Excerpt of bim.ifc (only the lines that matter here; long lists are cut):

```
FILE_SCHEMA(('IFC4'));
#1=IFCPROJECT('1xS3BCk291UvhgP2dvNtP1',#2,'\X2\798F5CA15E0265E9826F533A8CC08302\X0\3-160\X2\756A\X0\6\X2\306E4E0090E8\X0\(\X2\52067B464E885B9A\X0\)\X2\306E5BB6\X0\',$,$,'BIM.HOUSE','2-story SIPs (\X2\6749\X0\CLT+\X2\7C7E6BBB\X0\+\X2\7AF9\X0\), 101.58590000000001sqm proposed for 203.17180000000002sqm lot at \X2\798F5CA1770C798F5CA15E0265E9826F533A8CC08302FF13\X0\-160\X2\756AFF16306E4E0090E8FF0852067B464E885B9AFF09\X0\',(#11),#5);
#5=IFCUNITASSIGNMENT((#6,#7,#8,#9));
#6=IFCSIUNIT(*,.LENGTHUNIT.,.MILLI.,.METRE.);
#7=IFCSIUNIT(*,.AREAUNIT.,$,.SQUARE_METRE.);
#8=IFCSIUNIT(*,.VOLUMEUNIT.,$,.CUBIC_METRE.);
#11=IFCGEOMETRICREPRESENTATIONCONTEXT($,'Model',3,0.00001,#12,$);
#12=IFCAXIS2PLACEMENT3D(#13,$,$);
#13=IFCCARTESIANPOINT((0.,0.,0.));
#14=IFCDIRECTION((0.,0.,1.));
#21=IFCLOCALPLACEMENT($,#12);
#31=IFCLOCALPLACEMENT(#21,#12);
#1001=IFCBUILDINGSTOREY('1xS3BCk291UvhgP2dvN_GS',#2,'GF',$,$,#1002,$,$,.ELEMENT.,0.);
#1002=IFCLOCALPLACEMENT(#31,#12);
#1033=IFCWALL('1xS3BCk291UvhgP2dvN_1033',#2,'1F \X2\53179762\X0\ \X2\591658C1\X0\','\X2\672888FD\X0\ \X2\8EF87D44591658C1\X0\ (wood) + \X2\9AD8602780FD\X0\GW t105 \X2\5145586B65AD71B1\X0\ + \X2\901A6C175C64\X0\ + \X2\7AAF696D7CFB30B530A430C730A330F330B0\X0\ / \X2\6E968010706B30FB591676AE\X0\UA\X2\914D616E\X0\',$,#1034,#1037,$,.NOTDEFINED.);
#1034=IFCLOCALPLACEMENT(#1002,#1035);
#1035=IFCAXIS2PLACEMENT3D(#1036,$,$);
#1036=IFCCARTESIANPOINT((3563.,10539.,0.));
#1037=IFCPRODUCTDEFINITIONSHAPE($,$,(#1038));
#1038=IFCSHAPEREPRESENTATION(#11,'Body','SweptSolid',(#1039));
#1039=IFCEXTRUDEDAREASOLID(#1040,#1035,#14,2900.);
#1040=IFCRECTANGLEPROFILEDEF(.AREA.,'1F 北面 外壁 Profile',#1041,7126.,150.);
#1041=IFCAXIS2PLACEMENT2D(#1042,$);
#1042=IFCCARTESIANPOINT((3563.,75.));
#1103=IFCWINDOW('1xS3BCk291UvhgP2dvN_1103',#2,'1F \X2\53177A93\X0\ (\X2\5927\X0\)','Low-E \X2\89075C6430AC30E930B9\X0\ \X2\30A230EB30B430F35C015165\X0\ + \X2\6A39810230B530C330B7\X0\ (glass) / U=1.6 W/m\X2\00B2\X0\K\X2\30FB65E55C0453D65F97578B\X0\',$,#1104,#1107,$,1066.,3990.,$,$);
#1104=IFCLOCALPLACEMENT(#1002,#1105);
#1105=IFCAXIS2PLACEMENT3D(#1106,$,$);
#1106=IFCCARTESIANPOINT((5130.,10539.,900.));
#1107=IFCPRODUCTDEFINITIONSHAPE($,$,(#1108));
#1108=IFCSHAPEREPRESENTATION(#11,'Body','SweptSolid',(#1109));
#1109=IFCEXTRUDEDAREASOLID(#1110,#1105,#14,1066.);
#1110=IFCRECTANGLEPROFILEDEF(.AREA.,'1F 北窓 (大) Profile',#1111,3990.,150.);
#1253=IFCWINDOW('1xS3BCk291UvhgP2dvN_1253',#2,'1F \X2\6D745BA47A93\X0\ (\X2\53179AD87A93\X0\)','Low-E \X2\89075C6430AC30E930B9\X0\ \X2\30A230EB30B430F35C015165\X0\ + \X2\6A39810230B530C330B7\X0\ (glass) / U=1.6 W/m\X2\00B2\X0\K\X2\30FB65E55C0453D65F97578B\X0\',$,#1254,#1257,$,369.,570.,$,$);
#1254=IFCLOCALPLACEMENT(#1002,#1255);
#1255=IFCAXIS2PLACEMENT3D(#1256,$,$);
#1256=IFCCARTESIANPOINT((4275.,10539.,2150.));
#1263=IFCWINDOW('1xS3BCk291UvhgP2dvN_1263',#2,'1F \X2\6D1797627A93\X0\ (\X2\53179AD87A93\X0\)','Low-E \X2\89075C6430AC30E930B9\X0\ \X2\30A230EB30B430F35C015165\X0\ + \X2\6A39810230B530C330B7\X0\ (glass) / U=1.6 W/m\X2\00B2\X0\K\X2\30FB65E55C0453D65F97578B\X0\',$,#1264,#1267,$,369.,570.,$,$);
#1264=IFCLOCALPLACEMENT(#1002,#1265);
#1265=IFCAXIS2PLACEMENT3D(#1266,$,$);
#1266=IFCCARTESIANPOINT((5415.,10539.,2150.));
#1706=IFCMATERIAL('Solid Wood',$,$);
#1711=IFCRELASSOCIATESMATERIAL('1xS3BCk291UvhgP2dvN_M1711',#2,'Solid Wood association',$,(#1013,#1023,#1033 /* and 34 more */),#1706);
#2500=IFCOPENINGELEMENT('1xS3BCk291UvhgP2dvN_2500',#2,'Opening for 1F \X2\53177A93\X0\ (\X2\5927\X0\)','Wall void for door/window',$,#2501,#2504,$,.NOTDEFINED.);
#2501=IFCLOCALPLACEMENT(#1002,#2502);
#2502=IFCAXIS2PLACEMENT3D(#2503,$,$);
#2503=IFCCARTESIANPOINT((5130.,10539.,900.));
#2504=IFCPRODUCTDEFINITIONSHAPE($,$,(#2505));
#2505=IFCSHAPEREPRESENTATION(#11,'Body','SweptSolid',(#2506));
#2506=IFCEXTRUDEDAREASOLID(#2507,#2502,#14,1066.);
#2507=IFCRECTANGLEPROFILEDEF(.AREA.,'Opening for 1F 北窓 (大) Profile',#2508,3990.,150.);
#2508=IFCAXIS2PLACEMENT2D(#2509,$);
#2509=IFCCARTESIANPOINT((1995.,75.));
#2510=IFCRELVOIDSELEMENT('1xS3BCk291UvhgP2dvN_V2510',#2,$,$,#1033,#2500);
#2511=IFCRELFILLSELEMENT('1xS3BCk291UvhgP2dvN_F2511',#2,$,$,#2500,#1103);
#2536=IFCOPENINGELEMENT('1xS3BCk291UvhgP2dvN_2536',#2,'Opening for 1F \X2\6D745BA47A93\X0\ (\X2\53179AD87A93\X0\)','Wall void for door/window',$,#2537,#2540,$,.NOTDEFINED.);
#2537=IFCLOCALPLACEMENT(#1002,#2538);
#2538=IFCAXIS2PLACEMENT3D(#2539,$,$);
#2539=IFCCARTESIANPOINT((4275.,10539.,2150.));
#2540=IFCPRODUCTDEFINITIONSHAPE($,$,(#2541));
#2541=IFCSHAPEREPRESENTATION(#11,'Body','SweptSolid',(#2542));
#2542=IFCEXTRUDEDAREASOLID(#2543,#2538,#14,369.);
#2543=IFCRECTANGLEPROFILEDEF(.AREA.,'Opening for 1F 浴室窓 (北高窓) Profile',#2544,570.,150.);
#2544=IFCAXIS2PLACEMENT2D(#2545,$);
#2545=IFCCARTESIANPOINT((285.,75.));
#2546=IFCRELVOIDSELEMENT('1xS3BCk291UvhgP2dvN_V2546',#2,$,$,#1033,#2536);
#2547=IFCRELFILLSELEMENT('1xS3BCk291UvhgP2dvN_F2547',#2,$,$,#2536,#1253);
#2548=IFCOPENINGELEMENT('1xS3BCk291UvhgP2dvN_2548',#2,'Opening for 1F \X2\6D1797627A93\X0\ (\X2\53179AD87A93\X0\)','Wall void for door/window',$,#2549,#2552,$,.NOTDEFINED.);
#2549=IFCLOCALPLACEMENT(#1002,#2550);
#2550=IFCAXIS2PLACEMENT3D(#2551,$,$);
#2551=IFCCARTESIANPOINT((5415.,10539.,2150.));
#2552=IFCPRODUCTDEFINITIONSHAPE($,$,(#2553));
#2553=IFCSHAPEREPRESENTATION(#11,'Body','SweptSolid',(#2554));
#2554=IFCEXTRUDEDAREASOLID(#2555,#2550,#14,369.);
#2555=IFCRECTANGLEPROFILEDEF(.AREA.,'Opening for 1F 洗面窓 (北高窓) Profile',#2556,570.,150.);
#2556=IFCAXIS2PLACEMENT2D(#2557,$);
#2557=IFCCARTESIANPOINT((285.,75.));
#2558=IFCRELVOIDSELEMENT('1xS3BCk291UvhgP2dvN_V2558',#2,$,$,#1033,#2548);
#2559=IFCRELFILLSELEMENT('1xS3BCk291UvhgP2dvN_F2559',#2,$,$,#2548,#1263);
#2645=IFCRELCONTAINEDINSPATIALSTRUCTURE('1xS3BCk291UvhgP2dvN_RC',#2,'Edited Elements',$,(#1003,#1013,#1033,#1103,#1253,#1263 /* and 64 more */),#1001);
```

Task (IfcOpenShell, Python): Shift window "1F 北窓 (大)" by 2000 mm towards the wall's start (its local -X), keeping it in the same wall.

```python
import ifcopenshell
import ifcopenshell.api.geometry
import ifcopenshell.util.placement

model = ifcopenshell.open("bim.ifc")

window = model.by_guid("1xS3BCk291UvhgP2dvN_1103")
opening = window.FillsVoids[0].RelatingOpeningElement
wall = opening.VoidsElements[0].RelatingBuildingElement

wall_matrix = ifcopenshell.util.placement.get_local_placement(wall.ObjectPlacement)
shift = wall_matrix[:3, 0] * -2000.0
before = ifcopenshell.util.placement.get_local_placement(window.ObjectPlacement)[:3, 3].copy()

# The window is not placed relative to its opening, so move both.
for product in (opening, window):
    matrix = ifcopenshell.util.placement.get_local_placement(product.ObjectPlacement)
    matrix[:3, 3] += shift
    ifcopenshell.api.geometry.edit_object_placement(model, product=product, matrix=matrix, is_si=False)

after = ifcopenshell.util.placement.get_local_placement(window.ObjectPlacement)[:3, 3]
print("window moved by", (after - before).round(3) + 0.0)

model.write("bim_v2.ifc")
```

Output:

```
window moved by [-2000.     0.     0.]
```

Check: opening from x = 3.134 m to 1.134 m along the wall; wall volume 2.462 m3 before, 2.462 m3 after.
